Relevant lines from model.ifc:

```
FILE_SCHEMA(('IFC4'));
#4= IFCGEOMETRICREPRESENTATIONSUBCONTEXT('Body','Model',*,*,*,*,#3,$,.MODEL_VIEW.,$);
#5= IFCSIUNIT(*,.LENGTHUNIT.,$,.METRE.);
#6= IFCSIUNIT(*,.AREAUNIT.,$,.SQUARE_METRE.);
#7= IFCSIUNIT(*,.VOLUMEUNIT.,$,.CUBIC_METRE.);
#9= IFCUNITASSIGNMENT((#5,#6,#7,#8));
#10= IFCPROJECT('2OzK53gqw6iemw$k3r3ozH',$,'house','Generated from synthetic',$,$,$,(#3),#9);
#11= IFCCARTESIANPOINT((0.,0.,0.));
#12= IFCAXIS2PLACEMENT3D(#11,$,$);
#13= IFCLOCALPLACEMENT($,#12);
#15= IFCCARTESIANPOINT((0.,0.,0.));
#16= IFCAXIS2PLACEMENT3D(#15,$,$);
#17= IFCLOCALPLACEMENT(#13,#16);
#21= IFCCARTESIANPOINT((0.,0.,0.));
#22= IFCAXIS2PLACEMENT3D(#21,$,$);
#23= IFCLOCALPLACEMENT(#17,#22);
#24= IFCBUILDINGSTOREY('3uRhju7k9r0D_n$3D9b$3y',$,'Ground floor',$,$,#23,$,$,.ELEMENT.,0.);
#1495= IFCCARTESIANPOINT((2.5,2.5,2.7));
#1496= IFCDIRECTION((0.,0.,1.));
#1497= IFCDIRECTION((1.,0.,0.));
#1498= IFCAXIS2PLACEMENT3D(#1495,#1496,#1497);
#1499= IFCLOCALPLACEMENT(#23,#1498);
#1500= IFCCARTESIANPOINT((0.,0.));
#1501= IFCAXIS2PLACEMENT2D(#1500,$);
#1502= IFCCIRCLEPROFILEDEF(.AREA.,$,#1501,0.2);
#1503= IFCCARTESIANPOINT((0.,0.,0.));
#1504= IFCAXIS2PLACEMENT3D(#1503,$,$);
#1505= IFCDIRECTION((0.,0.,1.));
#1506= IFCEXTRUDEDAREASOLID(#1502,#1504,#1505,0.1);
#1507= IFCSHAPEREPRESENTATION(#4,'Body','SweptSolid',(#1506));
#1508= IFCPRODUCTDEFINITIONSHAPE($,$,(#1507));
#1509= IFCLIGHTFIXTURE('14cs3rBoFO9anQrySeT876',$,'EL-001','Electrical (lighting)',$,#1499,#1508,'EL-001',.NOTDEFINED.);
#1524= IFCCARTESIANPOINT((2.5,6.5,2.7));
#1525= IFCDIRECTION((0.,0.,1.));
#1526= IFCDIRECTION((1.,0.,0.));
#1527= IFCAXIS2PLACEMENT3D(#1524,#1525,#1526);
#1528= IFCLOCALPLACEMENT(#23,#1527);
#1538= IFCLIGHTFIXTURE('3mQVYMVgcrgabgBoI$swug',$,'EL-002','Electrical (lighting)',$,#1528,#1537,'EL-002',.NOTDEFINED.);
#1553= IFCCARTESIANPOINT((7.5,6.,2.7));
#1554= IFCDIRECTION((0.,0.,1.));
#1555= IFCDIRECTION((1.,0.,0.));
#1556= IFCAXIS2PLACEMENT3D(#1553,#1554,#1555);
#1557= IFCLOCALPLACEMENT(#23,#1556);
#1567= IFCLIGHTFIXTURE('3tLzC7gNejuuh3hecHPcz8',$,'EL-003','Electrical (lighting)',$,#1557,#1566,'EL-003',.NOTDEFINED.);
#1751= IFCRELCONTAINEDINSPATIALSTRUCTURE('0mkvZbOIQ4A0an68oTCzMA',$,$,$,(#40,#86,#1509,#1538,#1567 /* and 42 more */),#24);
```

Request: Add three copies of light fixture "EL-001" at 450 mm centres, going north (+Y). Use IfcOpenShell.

```python
import numpy as np
import ifcopenshell
import ifcopenshell.api.geometry
import ifcopenshell.api.root
import ifcopenshell.util.element
import ifcopenshell.util.placement
import ifcopenshell.util.unit

model = ifcopenshell.open("model.ifc")
unit_scale = ifcopenshell.util.unit.calculate_unit_scale(model)

source = model.by_guid("14cs3rBoFO9anQrySeT876")
base = ifcopenshell.util.placement.get_local_placement(source.ObjectPlacement)
step = np.array([0.0, 1.0, 0.0]) * 0.45 / unit_scale

for i in range(1, 4):
    copy = ifcopenshell.api.root.copy_class(model, product=source)
    copy.Representation = ifcopenshell.util.element.copy_deep(
        model, source.Representation, exclude=["IfcGeometricRepresentationContext", "IfcRepresentationMap"]
    )
    copy.Tag = None
    matrix = base.copy()
    matrix[:3, 3] += i * step
    print("added at", matrix[:3, 3].round(3) + 0.0)
    ifcopenshell.api.geometry.edit_object_placement(model, product=copy, matrix=matrix, is_si=False)

model.write("model_v2.ifc")
```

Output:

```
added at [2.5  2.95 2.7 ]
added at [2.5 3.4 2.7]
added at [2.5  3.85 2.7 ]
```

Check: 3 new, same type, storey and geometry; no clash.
